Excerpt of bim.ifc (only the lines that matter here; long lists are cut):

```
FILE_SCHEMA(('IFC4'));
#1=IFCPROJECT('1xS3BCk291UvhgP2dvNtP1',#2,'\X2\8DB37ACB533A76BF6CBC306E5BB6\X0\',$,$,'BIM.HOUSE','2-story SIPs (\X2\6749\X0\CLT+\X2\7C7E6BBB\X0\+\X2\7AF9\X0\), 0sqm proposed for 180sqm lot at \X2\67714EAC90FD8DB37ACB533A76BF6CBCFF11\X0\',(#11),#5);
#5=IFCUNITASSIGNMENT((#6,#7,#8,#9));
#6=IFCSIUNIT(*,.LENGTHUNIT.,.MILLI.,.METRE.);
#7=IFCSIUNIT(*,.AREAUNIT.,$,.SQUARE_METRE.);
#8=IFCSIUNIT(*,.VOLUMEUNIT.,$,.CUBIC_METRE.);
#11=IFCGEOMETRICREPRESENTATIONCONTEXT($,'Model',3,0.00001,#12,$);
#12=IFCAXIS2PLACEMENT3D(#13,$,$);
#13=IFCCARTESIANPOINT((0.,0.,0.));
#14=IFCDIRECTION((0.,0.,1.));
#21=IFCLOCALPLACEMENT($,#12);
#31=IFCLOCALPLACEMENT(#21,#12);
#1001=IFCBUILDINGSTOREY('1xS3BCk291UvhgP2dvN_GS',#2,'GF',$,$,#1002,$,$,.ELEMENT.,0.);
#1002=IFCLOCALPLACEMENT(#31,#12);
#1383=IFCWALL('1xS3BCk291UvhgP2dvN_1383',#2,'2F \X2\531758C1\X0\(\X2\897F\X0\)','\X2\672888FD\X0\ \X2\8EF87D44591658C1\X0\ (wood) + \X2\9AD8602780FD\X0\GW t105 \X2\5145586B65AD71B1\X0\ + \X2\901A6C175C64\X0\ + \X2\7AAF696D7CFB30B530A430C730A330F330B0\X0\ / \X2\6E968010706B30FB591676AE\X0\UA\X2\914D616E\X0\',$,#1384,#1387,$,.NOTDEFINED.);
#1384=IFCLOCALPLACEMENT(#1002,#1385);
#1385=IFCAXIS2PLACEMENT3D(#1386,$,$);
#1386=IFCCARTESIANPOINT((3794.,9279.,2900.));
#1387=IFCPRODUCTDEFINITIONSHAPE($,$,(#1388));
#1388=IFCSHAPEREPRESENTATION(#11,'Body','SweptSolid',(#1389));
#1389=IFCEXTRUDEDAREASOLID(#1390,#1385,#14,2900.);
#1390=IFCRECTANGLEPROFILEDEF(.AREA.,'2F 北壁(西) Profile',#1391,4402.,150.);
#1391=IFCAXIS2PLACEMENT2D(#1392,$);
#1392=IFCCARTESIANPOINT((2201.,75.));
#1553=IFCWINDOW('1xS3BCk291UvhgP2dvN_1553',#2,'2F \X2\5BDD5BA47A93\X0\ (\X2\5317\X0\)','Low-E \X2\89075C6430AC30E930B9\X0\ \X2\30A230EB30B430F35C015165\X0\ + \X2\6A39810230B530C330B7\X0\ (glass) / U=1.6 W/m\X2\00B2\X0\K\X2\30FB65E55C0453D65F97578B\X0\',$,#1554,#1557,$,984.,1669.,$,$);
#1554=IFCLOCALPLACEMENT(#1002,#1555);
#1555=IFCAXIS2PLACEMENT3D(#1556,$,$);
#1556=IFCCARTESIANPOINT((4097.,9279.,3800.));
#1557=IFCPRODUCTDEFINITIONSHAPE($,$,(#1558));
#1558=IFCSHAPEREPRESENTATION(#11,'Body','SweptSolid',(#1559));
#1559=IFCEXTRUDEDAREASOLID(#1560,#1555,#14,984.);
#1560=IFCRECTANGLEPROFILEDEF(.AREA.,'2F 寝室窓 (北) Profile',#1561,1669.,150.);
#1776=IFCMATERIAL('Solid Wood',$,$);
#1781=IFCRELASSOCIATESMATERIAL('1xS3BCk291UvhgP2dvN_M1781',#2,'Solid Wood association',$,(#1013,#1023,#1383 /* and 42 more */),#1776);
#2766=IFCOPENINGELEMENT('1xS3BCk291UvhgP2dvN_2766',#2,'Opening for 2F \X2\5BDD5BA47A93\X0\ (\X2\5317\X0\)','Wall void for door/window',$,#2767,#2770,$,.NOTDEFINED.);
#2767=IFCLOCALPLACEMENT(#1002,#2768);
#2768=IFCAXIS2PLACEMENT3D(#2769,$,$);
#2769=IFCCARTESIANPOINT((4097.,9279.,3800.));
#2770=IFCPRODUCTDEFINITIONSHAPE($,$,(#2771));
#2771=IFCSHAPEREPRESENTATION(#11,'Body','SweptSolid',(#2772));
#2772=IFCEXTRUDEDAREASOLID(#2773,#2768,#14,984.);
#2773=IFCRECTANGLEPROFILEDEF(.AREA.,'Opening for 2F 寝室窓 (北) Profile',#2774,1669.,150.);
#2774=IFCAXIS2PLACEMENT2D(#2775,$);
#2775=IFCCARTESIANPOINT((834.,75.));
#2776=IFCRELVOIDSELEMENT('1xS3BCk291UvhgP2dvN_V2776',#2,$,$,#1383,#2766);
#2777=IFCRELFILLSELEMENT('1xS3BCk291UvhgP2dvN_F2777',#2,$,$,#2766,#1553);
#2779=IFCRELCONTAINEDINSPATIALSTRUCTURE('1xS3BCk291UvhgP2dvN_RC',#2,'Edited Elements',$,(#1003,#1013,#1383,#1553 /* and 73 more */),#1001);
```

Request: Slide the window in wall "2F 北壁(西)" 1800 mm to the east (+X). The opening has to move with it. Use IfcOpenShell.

```python
import ifcopenshell
import ifcopenshell.api.geometry
import ifcopenshell.util.placement

model = ifcopenshell.open("bim.ifc")

window = model.by_id(1553)
opening = window.FillsVoids[0].RelatingOpeningElement
wall = opening.VoidsElements[0].RelatingBuildingElement

wall_matrix = ifcopenshell.util.placement.get_local_placement(wall.ObjectPlacement)
shift = wall_matrix[:3, 0] * 1800.0
before = ifcopenshell.util.placement.get_local_placement(window.ObjectPlacement)[:3, 3].copy()

# The window is not placed relative to its opening, so move both.
for product in (opening, window):
    matrix = ifcopenshell.util.placement.get_local_placement(product.ObjectPlacement)
    matrix[:3, 3] += shift
    ifcopenshell.api.geometry.edit_object_placement(model, product=product, matrix=matrix, is_si=False)

after = ifcopenshell.util.placement.get_local_placement(window.ObjectPlacement)[:3, 3]
print("window moved by", (after - before).round(3) + 0.0)

model.write("bim_updated.ifc")
```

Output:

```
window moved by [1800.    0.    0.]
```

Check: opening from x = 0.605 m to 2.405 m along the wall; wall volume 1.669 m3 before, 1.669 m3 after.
